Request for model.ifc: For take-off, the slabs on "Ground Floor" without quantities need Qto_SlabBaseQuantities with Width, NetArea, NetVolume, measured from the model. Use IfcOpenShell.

First a look at what the model holds.

```python
import ifcopenshell
import ifcopenshell.util.element
import ifcopenshell.util.unit

model = ifcopenshell.open("model.ifc")
print(model.schema)
for unit_type in ("LENGTHUNIT", "AREAUNIT", "VOLUMEUNIT"):
    print(unit_type, ifcopenshell.util.unit.calculate_unit_scale(model, unit_type))
storey = next(s for s in model.by_type("IfcBuildingStorey") if s.Name == "Ground Floor")
slabs = [e for e in ifcopenshell.util.element.get_decomposition(storey) if e.is_a("IfcSlab")]
for e in sorted(slabs, key=lambda e: e.id()):
    print(e.id(), e.is_a(), e.Name, list(ifcopenshell.util.element.get_psets(e, qtos_only=True)), sep=" | ")
```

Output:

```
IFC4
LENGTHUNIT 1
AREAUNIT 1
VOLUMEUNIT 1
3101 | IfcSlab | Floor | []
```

```python
import ifcopenshell
import ifcopenshell.api.pset
import ifcopenshell.geom
import ifcopenshell.util.element
import ifcopenshell.util.shape
import ifcopenshell.util.unit

model = ifcopenshell.open("model.ifc")
unit_scale = ifcopenshell.util.unit.calculate_unit_scale(model)
area_scale = ifcopenshell.util.unit.calculate_unit_scale(model, "AREAUNIT")
volume_scale = ifcopenshell.util.unit.calculate_unit_scale(model, "VOLUMEUNIT")
settings = ifcopenshell.geom.settings()

storey = next(s for s in model.by_type("IfcBuildingStorey") if s.Name == "Ground Floor")
slabs = [e for e in ifcopenshell.util.element.get_decomposition(storey) if e.is_a("IfcSlab")]

for e in sorted(slabs, key=lambda e: e.id()):
    if ifcopenshell.util.element.get_psets(e, qtos_only=True, should_inherit=False):
        continue
    # Geometry comes back in metres, in the element's own axes.
    shape = ifcopenshell.geom.create_shape(settings, e)
    values = {
        "Width": ifcopenshell.util.shape.get_z(shape.geometry) / unit_scale,
        "NetArea": ifcopenshell.util.shape.get_footprint_area(shape.geometry) / area_scale,
        "NetVolume": ifcopenshell.util.shape.get_volume(shape.geometry) / volume_scale,
    }
    qto = ifcopenshell.api.pset.add_qto(model, product=e, name="Qto_SlabBaseQuantities")
    ifcopenshell.api.pset.edit_qto(model, qto=qto, properties=values)
    print(e.id(), {k: round(v, 3) for k, v in values.items()})

model.write("model_edited.ifc")
```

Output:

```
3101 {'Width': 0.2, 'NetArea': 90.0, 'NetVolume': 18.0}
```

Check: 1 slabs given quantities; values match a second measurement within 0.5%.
